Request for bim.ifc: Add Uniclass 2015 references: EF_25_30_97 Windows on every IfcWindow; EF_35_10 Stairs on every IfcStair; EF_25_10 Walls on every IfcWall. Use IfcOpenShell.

First a look at what the model holds.

```python
import ifcopenshell

model = ifcopenshell.open("bim.ifc")
print(model.schema)
print("classifications:", [c.Name for c in model.by_type("IfcClassification")])
for ifc_class in ("IfcDoor", "IfcRoof", "IfcStair", "IfcWall", "IfcWindow"):
    print(ifc_class, len(model.by_type(ifc_class)))
```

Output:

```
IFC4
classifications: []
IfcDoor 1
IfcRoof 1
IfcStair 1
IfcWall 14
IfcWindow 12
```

```python
import ifcopenshell
import ifcopenshell.api.classification

model = ifcopenshell.open("bim.ifc")

system = ifcopenshell.api.classification.add_classification(model, classification="Uniclass 2015")

codes = {
    "IfcWindow": ("EF_25_30_97", "Windows"),
    "IfcStair": ("EF_35_10", "Stairs"),
    "IfcWall": ("EF_25_10", "Walls"),
}
for ifc_class, (code, name) in codes.items():
    products = model.by_type(ifc_class)
    ifcopenshell.api.classification.add_reference(
        model, products=products, classification=system, identification=code, name=name
    )
    print(code, len(products))

model.write("bim-out.ifc")
```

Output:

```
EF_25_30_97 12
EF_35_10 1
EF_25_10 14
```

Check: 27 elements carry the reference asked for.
